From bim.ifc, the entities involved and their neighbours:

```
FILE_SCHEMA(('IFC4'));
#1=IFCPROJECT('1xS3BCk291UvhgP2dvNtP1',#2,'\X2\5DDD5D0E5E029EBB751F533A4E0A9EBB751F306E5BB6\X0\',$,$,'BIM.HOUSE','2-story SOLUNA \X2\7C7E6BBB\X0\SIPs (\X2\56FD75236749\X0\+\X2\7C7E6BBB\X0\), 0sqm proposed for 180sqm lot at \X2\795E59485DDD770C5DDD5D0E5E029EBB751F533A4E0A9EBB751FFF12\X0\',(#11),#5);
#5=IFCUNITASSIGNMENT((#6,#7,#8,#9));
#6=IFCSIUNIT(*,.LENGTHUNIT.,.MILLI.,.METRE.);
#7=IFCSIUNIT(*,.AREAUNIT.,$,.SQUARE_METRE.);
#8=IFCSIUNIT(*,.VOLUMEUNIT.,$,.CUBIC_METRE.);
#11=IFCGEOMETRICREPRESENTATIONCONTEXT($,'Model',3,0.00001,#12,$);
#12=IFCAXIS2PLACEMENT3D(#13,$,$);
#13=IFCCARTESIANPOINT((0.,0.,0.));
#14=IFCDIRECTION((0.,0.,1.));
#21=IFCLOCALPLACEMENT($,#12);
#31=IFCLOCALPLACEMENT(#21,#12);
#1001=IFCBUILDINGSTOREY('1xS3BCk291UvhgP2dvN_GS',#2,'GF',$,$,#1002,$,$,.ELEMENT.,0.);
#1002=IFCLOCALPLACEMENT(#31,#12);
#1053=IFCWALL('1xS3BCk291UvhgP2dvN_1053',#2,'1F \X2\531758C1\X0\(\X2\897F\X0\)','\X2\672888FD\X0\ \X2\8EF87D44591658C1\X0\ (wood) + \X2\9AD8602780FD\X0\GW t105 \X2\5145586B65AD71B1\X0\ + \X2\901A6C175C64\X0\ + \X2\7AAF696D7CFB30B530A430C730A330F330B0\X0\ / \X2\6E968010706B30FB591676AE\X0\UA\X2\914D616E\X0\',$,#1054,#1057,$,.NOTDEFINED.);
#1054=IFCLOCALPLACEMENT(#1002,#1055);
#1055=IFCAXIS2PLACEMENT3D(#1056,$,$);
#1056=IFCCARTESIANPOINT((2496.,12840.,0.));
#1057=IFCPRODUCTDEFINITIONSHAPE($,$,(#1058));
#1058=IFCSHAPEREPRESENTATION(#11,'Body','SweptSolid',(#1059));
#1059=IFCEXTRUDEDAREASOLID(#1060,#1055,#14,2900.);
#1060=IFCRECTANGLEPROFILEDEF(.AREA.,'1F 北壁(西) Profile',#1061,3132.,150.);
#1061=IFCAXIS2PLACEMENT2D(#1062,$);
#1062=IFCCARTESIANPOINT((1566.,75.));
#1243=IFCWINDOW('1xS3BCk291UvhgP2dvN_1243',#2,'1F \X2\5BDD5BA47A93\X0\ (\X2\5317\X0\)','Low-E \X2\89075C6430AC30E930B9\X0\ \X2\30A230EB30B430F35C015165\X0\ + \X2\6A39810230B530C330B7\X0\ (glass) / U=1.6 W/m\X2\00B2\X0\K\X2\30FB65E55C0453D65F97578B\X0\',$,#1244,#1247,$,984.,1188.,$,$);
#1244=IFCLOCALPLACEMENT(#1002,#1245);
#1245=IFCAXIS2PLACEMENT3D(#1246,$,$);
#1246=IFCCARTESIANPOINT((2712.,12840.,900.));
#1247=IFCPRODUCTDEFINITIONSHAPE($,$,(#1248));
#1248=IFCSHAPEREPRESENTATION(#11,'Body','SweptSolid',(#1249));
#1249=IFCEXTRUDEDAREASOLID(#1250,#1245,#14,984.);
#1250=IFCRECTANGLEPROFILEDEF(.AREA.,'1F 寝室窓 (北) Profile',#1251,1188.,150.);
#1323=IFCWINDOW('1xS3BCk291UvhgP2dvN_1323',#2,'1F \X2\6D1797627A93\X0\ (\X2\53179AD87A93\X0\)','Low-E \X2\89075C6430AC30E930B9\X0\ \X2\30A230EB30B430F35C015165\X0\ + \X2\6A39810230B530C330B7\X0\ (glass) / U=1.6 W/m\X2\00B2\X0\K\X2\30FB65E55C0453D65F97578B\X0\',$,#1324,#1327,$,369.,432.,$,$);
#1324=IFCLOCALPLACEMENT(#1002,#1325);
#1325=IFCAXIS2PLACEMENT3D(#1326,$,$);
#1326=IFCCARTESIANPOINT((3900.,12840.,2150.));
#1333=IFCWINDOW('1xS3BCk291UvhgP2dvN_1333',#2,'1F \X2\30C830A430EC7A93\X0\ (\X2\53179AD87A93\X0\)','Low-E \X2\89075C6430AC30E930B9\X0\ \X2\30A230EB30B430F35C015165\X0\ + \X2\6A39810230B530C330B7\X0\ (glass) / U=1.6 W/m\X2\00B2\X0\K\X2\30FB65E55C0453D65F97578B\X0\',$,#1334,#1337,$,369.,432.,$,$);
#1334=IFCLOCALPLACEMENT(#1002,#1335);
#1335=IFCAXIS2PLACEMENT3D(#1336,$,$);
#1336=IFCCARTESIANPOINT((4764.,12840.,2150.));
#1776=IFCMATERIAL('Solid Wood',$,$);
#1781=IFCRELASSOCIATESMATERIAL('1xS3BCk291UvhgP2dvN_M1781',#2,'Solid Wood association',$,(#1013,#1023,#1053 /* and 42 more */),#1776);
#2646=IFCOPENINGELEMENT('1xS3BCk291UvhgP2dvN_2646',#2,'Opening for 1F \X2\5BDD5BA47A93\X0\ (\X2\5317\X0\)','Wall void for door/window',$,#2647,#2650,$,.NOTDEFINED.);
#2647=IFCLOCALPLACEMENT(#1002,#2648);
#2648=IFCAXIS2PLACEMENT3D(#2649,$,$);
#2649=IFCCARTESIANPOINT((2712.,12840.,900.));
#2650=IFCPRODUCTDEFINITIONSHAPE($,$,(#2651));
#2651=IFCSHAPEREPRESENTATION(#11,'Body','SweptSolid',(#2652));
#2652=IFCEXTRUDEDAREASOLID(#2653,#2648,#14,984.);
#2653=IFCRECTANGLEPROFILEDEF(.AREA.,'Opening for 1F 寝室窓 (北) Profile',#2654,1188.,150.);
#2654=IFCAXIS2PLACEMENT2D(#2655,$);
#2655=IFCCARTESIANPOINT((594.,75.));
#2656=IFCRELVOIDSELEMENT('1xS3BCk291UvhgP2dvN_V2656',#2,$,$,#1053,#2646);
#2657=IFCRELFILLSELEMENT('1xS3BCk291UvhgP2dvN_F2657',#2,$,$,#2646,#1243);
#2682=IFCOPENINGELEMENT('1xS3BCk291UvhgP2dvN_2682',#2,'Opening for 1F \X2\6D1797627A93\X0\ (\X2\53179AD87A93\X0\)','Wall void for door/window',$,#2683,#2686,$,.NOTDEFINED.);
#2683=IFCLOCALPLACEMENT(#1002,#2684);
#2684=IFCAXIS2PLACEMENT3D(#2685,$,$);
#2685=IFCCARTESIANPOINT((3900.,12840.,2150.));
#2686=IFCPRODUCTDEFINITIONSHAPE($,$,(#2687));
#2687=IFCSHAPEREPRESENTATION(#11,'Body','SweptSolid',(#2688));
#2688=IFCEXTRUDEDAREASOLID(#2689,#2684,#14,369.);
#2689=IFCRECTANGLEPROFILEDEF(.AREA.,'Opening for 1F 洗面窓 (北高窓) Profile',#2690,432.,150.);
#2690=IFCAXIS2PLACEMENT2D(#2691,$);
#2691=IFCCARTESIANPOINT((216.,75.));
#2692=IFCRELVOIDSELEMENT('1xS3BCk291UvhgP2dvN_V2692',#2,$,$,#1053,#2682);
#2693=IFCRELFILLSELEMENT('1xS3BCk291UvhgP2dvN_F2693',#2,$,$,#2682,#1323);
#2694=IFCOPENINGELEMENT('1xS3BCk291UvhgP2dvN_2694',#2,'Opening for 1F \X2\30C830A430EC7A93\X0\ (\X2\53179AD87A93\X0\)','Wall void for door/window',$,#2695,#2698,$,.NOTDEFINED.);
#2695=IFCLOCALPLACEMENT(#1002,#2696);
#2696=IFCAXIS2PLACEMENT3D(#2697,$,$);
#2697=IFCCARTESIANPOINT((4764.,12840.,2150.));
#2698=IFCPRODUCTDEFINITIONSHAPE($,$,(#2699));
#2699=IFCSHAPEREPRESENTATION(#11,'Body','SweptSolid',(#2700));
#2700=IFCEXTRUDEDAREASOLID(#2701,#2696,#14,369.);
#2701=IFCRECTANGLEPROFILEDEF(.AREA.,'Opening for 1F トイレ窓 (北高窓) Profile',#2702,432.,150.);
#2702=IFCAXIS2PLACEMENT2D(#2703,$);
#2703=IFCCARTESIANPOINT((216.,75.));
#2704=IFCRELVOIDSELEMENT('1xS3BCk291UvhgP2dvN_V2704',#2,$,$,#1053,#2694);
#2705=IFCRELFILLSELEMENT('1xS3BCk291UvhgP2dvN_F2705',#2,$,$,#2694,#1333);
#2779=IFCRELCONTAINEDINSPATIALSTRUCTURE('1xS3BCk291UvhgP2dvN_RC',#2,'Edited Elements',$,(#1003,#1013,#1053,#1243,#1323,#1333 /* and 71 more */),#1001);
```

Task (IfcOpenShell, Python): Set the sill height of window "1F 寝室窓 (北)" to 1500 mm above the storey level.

```python
import numpy as np
import ifcopenshell
import ifcopenshell.api.geometry
import ifcopenshell.geom
import ifcopenshell.util.element
import ifcopenshell.util.placement
import ifcopenshell.util.shape
import ifcopenshell.util.unit

model = ifcopenshell.open("bim.ifc")
unit_scale = ifcopenshell.util.unit.calculate_unit_scale(model)

window = model.by_guid("1xS3BCk291UvhgP2dvN_1243")
opening = window.FillsVoids[0].RelatingOpeningElement
storey = ifcopenshell.util.element.get_container(window, ifc_class="IfcBuildingStorey")
level = ifcopenshell.util.placement.get_local_placement(storey.ObjectPlacement)[2, 3]

# The opening's origin need not be at the sill, so measure its lowest point.
shape = ifcopenshell.geom.create_shape(ifcopenshell.geom.settings(), opening)
bottom = ifcopenshell.util.shape.get_shape_bottom_elevation(shape, shape.geometry) / unit_scale
dz = level + 1500.0 - bottom

shift = np.array([0.0, 0.0, dz])
# The window is not placed relative to its opening, so move both.
for product in (opening, window):
    matrix = ifcopenshell.util.placement.get_local_placement(product.ObjectPlacement)
    matrix[:3, 3] += shift
    ifcopenshell.api.geometry.edit_object_placement(model, product=product, matrix=matrix, is_si=False)

print(f"moved by {dz * unit_scale:+.3f} m")

model.write("bim-out.ifc")
```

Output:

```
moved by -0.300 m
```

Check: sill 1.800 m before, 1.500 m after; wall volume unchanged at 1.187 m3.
